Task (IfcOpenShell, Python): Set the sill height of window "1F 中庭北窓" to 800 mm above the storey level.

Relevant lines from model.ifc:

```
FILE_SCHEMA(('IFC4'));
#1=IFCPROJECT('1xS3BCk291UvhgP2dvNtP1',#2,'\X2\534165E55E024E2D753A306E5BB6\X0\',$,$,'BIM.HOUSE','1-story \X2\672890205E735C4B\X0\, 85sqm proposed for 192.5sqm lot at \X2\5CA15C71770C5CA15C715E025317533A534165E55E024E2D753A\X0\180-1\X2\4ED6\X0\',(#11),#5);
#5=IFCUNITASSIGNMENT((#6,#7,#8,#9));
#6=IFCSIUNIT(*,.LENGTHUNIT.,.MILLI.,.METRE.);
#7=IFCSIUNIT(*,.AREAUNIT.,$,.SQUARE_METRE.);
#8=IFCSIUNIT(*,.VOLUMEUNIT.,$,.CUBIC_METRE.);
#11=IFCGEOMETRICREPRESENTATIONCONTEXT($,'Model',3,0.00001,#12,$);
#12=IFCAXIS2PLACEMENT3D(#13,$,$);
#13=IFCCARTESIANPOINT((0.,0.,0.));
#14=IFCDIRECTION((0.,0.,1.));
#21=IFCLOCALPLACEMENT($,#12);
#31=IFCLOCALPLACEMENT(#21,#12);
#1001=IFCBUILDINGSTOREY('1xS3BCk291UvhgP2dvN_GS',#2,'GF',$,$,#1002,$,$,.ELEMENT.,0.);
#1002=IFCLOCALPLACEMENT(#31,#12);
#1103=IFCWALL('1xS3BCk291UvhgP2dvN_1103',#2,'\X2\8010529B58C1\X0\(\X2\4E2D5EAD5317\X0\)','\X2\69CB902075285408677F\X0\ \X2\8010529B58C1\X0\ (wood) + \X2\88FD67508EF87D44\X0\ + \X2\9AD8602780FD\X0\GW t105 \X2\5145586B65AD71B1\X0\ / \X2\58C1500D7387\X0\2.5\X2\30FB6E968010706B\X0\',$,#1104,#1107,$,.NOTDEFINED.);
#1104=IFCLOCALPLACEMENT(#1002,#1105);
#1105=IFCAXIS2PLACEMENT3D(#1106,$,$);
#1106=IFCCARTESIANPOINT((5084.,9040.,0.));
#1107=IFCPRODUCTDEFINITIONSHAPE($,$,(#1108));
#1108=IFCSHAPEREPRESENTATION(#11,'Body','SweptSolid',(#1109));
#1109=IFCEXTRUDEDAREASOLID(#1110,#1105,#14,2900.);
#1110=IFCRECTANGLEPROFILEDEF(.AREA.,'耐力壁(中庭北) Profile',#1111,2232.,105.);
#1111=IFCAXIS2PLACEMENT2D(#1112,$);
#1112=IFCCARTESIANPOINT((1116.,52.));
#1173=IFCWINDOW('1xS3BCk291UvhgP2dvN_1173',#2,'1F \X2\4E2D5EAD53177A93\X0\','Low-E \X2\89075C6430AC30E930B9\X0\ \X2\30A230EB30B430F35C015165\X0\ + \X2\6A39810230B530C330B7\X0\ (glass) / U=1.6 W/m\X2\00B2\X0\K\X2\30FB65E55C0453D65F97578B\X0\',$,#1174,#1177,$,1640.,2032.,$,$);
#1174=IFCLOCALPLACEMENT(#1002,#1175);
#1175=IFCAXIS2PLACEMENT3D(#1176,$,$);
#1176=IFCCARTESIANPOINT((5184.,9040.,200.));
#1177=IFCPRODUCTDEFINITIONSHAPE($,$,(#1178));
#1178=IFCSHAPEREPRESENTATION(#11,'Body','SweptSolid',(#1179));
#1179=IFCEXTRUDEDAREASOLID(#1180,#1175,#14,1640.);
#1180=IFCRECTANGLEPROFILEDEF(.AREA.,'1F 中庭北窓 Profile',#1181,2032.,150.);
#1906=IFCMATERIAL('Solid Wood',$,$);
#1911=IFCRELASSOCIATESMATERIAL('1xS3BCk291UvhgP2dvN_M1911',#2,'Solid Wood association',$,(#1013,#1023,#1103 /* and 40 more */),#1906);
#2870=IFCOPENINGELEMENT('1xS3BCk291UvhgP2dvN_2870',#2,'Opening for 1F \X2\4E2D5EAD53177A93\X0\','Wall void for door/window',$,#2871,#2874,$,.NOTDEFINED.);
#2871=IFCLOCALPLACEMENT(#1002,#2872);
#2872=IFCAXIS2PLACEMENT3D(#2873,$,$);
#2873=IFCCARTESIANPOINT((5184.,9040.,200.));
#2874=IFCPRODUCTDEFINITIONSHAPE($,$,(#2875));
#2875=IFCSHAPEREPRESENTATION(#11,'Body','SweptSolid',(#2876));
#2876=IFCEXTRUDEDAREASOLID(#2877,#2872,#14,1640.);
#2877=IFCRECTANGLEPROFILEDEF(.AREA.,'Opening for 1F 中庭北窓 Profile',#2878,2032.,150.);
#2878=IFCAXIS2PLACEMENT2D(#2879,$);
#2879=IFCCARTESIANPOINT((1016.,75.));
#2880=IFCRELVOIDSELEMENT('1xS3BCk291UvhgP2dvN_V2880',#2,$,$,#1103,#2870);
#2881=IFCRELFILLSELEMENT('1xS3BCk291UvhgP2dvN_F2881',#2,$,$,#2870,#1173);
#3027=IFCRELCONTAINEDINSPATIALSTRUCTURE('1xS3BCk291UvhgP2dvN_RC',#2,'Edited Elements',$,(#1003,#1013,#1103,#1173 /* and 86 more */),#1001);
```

```python
import numpy as np
import ifcopenshell
import ifcopenshell.api.geometry
import ifcopenshell.geom
import ifcopenshell.util.element
import ifcopenshell.util.placement
import ifcopenshell.util.shape
import ifcopenshell.util.unit

model = ifcopenshell.open("model.ifc")
unit_scale = ifcopenshell.util.unit.calculate_unit_scale(model)

window = model.by_guid("1xS3BCk291UvhgP2dvN_1173")
opening = window.FillsVoids[0].RelatingOpeningElement
storey = ifcopenshell.util.element.get_container(window, ifc_class="IfcBuildingStorey")
level = ifcopenshell.util.placement.get_local_placement(storey.ObjectPlacement)[2, 3]

# The opening's origin need not be at the sill, so measure its lowest point.
shape = ifcopenshell.geom.create_shape(ifcopenshell.geom.settings(), opening)
bottom = ifcopenshell.util.shape.get_shape_bottom_elevation(shape, shape.geometry) / unit_scale
dz = level + 0.8 / unit_scale - bottom

shift = np.array([0.0, 0.0, dz])
# The window is not placed relative to its opening, so move both.
for product in (opening, window):
    matrix = ifcopenshell.util.placement.get_local_placement(product.ObjectPlacement)
    matrix[:3, 3] += shift
    ifcopenshell.api.geometry.edit_object_placement(model, product=product, matrix=matrix, is_si=False)

print(f"moved by {dz * unit_scale:+.3f} m")

model.write("model_rev.ifc")
```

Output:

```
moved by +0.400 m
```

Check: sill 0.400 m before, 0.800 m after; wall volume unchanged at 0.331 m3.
